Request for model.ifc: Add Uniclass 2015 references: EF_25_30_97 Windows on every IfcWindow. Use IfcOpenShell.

First a look at what the model holds.

```python
import ifcopenshell

model = ifcopenshell.open("model.ifc")
print(model.schema)
print("classifications:", [c.Name for c in model.by_type("IfcClassification")])
for ifc_class in ("IfcDoor", "IfcRoof", "IfcStair", "IfcWall", "IfcWindow"):
    print(ifc_class, len(model.by_type(ifc_class)))
```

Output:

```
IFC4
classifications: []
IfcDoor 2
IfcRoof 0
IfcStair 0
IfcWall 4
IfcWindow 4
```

```python
import ifcopenshell
import ifcopenshell.api.classification

model = ifcopenshell.open("model.ifc")

system = ifcopenshell.api.classification.add_classification(model, classification="Uniclass 2015")

codes = {
    "IfcWindow": ("EF_25_30_97", "Windows"),
}
for ifc_class, (code, name) in codes.items():
    products = model.by_type(ifc_class)
    ifcopenshell.api.classification.add_reference(
        model, products=products, classification=system, identification=code, name=name
    )
    print(code, len(products))

model.write("model_v2.ifc")
```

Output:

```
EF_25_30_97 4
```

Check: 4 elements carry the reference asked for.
